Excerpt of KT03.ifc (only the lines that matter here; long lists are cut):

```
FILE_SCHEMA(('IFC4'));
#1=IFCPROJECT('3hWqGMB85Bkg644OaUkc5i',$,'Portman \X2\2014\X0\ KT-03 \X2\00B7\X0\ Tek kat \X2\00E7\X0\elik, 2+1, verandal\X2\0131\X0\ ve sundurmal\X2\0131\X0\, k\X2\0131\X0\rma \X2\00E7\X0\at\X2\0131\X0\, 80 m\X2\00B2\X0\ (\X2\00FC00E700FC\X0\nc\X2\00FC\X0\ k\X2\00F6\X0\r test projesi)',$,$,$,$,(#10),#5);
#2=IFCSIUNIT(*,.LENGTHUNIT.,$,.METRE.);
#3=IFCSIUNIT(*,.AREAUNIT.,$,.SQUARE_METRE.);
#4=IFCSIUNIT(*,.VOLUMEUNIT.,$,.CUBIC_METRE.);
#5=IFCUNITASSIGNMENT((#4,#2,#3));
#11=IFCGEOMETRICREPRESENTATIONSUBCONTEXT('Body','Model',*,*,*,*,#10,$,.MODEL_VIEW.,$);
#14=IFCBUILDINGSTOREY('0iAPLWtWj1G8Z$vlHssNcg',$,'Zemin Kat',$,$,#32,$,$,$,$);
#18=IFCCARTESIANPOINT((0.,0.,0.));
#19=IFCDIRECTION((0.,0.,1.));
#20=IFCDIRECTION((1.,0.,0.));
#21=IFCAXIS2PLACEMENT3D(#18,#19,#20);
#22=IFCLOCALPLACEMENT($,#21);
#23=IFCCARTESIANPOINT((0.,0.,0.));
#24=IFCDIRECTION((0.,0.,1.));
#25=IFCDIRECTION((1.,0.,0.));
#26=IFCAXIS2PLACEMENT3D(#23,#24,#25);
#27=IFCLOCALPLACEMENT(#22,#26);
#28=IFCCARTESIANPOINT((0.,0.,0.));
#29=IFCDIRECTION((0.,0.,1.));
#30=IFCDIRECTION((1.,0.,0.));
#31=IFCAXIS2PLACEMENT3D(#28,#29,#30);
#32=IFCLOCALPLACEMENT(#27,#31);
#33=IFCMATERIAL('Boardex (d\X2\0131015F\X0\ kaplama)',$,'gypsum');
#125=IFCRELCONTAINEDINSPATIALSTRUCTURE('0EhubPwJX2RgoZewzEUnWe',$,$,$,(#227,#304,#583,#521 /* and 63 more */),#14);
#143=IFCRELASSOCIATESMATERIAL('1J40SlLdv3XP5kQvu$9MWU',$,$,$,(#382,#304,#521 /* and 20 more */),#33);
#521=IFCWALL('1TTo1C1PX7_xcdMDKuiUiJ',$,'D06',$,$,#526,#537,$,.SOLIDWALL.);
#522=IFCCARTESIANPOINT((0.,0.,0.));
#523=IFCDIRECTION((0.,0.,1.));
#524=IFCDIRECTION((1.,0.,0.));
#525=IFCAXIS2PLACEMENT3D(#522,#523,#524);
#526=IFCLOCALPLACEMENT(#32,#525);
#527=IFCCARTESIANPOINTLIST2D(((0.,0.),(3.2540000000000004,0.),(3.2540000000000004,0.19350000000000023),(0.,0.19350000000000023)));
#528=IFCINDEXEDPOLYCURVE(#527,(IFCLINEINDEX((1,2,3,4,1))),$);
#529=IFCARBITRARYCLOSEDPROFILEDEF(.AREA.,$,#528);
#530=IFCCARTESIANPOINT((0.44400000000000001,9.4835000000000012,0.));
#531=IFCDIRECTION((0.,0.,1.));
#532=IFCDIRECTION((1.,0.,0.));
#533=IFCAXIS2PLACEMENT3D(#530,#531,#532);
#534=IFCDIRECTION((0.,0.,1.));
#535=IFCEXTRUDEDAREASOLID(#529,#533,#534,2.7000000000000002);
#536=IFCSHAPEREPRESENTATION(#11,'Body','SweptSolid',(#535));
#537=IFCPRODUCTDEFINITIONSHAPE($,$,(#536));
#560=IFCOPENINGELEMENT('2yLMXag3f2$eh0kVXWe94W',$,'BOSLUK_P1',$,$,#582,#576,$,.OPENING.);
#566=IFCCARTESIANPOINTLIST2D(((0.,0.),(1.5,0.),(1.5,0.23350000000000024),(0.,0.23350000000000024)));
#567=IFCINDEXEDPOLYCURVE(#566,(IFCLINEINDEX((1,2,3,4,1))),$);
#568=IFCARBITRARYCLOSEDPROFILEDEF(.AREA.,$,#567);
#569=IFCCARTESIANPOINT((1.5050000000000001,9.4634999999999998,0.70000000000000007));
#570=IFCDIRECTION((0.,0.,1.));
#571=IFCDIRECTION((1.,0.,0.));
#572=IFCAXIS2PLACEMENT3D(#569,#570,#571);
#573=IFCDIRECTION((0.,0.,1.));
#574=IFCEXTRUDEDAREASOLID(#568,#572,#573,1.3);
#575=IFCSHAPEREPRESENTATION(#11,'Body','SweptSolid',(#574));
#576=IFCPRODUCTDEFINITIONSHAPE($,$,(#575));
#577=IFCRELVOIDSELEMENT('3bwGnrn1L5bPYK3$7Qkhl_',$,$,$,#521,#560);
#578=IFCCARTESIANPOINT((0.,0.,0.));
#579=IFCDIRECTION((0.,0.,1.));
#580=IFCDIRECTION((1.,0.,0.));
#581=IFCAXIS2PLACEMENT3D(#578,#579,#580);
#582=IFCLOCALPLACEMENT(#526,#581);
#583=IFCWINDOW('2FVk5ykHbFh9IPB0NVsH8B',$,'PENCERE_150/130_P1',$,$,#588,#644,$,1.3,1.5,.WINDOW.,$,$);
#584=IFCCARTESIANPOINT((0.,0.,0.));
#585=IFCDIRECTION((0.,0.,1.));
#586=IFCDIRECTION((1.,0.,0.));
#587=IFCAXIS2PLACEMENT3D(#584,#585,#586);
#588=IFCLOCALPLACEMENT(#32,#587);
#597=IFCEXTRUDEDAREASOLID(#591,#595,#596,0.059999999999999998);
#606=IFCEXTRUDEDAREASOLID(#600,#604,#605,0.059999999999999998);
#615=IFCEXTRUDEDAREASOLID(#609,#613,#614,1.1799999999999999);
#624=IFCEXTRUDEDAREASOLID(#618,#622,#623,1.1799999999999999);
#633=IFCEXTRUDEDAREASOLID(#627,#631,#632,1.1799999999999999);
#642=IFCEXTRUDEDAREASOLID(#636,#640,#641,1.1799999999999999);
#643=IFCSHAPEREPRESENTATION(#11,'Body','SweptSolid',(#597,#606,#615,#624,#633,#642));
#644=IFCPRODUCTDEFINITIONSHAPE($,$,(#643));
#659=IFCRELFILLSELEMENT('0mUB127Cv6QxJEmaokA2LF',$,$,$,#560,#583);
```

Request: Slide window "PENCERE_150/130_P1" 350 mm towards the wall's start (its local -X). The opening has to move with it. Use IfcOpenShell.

```python
import ifcopenshell
import ifcopenshell.api.geometry
import ifcopenshell.util.placement
import ifcopenshell.util.unit

model = ifcopenshell.open("KT03.ifc")
unit_scale = ifcopenshell.util.unit.calculate_unit_scale(model)

window = model.by_guid("2FVk5ykHbFh9IPB0NVsH8B")
opening = window.FillsVoids[0].RelatingOpeningElement
wall = opening.VoidsElements[0].RelatingBuildingElement

wall_matrix = ifcopenshell.util.placement.get_local_placement(wall.ObjectPlacement)
shift = wall_matrix[:3, 0] * -0.35 / unit_scale
before = ifcopenshell.util.placement.get_local_placement(window.ObjectPlacement)[:3, 3].copy()

# The window is not placed relative to its opening, so move both.
for product in (opening, window):
    matrix = ifcopenshell.util.placement.get_local_placement(product.ObjectPlacement)
    matrix[:3, 3] += shift
    ifcopenshell.api.geometry.edit_object_placement(model, product=product, matrix=matrix, is_si=False)

after = ifcopenshell.util.placement.get_local_placement(window.ObjectPlacement)[:3, 3]
print("window moved by", (after - before).round(3) + 0.0)

model.write("KT03-out.ifc")
```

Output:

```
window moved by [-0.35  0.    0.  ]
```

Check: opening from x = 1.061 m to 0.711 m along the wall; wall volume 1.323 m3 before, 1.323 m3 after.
